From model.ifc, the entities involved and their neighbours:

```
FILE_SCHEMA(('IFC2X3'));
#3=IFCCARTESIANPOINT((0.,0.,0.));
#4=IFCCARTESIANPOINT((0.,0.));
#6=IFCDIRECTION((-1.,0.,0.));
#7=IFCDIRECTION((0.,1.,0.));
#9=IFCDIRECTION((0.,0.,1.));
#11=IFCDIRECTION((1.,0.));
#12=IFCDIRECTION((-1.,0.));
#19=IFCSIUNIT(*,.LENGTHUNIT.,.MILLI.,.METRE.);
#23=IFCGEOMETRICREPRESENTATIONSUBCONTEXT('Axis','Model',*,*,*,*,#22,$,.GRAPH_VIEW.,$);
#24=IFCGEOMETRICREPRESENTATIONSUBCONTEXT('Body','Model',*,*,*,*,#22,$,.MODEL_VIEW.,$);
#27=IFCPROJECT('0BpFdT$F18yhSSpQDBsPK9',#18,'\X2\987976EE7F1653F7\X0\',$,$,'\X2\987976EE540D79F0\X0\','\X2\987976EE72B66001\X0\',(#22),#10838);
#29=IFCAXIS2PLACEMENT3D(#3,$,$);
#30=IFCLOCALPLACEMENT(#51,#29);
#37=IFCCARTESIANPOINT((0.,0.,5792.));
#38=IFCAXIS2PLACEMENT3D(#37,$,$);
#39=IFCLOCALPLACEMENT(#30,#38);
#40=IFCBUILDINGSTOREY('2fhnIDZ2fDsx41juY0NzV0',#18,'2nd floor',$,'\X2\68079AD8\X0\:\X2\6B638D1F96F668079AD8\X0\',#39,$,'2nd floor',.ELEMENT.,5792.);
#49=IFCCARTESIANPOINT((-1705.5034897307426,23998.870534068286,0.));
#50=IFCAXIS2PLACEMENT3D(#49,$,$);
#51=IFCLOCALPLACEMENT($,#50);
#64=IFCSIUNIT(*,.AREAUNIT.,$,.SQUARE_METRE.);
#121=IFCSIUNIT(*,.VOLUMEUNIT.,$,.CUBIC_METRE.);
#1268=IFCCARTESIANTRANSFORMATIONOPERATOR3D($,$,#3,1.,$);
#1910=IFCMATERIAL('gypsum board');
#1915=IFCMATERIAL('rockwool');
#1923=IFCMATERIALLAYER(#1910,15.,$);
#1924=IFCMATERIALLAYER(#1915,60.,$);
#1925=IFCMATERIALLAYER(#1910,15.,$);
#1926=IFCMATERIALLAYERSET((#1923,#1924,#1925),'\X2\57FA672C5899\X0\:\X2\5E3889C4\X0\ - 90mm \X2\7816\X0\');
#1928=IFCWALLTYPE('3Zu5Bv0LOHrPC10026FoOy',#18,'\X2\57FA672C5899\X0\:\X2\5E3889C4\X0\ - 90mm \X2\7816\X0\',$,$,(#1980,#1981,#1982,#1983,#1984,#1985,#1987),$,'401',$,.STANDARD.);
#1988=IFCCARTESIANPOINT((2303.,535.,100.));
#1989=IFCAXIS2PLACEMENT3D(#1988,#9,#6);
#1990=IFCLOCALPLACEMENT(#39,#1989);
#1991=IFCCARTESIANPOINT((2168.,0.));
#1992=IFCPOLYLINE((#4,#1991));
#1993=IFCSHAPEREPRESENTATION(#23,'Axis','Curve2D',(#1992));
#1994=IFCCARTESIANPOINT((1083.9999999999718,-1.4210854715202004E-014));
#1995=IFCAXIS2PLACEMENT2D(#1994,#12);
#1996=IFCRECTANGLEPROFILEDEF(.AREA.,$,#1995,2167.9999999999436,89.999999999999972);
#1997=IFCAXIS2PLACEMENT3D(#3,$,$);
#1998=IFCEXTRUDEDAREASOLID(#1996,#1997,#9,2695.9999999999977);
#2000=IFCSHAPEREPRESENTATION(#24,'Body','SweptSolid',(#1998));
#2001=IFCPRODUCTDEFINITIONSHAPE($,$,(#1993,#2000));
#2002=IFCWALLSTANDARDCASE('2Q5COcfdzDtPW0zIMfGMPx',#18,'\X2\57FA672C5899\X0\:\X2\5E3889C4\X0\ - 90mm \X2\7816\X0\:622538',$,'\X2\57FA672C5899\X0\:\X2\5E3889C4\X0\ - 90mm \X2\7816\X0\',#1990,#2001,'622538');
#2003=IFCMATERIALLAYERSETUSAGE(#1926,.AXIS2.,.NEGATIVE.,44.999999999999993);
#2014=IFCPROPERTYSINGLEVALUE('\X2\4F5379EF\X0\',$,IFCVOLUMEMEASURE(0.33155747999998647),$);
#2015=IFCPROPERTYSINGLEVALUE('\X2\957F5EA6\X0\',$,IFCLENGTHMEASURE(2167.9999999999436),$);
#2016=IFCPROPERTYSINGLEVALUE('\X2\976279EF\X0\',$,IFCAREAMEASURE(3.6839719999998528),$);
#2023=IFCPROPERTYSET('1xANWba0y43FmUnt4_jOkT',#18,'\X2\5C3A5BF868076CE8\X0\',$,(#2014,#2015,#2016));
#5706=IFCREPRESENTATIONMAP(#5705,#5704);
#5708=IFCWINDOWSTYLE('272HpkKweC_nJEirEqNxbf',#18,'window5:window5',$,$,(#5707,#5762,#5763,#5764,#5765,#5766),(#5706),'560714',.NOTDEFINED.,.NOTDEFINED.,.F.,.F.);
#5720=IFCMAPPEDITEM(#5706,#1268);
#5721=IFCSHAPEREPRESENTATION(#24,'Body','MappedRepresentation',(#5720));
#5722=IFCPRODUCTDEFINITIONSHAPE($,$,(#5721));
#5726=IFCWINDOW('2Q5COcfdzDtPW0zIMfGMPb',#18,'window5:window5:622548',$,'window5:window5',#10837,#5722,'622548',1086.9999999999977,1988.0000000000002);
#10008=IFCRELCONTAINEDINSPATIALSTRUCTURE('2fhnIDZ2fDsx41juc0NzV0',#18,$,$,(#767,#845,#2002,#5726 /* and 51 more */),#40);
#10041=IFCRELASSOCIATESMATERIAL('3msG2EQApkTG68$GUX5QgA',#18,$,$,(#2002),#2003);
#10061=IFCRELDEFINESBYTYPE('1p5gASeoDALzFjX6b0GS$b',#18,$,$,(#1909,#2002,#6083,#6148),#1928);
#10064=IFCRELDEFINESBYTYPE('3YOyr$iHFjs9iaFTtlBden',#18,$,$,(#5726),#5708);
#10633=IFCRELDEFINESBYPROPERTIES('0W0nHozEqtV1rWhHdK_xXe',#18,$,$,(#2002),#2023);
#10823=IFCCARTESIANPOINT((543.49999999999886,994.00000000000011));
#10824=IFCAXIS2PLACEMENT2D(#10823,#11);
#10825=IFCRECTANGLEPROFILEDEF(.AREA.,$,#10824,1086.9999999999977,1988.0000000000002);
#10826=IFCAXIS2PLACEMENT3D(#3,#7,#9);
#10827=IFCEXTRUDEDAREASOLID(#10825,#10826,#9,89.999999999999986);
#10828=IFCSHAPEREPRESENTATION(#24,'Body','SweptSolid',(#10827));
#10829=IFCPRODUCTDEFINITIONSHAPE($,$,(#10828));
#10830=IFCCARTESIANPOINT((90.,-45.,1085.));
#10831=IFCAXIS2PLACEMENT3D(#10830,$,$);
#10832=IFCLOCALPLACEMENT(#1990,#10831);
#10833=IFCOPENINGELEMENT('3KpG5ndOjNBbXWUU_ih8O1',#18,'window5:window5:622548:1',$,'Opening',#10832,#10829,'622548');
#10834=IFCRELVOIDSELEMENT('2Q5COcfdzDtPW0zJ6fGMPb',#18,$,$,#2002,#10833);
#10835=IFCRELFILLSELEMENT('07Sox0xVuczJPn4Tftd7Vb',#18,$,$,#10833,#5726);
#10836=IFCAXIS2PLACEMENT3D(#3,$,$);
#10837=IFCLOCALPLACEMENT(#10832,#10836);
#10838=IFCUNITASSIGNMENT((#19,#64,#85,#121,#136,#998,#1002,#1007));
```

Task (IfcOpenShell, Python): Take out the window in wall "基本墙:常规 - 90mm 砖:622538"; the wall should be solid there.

```python
import ifcopenshell
import ifcopenshell.api.feature
import ifcopenshell.api.pset
import ifcopenshell.api.root
import ifcopenshell.geom
import ifcopenshell.util.element
import ifcopenshell.util.shape
import ifcopenshell.util.unit

model = ifcopenshell.open("model.ifc")
area_scale = ifcopenshell.util.unit.calculate_unit_scale(model, "AREAUNIT")
volume_scale = ifcopenshell.util.unit.calculate_unit_scale(model, "VOLUMEUNIT")
settings = ifcopenshell.geom.settings()


def volume(element):
    """Net volume in cubic metres, openings subtracted."""
    shape = ifcopenshell.geom.create_shape(settings, element)
    return ifcopenshell.util.shape.get_volume(shape.geometry)


window = model.by_guid("2Q5COcfdzDtPW0zIMfGMPb")
opening = window.FillsVoids[0].RelatingOpeningElement
wall = opening.VoidsElements[0].RelatingBuildingElement
before = volume(wall)

ifcopenshell.api.root.remove_product(model, product=window)
ifcopenshell.api.feature.remove_feature(model, feature=opening)

after = volume(wall)
thickness = 0.09  # wall thickness in metres

# Update the wall's stored quantities.
pset = model.by_id(ifcopenshell.util.element.get_pset(wall, "尺寸标注", should_inherit=False)["id"])
ifcopenshell.api.pset.edit_pset(model, pset=pset, properties={
    "体积": model.create_entity("IfcVolumeMeasure", after / volume_scale),
    "面积": model.create_entity("IfcAreaMeasure", after / thickness / area_scale),
})

print(f"wall volume {before:.3f} -> {after:.3f} m3")

model.write("model_v2.ifc")
```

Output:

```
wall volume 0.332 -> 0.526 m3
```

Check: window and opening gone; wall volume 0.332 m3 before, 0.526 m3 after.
